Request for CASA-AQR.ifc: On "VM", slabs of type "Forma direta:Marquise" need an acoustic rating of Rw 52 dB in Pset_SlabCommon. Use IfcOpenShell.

First a look at what the model holds.

```python
import ifcopenshell
import ifcopenshell.util.element

model = ifcopenshell.open("CASA-AQR.ifc")
print(model.schema)
storey = next(s for s in model.by_type("IfcBuildingStorey") if s.Name == "VM")
slabs = [e for e in ifcopenshell.util.element.get_decomposition(storey) if e.is_a("IfcSlab")]
seen = {}
for e in slabs:
    element_type = ifcopenshell.util.element.get_type(e)
    key = (element_type.Name if element_type != e and element_type else None, ifcopenshell.util.element.get_pset(e, "Pset_SlabCommon", "AcousticRating"))
    seen[key] = seen.get(key, 0) + 1
for (name, value), count in sorted(seen.items(), key=str):
    print(count, "x", name, "|", value)
```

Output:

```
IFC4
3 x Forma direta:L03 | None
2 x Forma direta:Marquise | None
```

```python
import ifcopenshell
import ifcopenshell.api.pset
import ifcopenshell.util.element

model = ifcopenshell.open("CASA-AQR.ifc")

storey = next(s for s in model.by_type("IfcBuildingStorey") if s.Name == "VM")
slabs = [e for e in ifcopenshell.util.element.get_decomposition(storey) if e.is_a("IfcSlab")]

count = 0
for e in slabs:
    element_type = ifcopenshell.util.element.get_type(e)
    if element_type in (None, e) or element_type.Name != "Forma direta:Marquise":
        continue
    # add_pset returns the element's existing set when there is one.
    pset = ifcopenshell.api.pset.add_pset(model, product=e, name="Pset_SlabCommon")
    ifcopenshell.api.pset.edit_pset(model, pset=pset, properties={"AcousticRating": "Rw 52 dB"})
    count += 1

print(count, "slabs updated")

model.write("CASA-AQR_v2.ifc")
```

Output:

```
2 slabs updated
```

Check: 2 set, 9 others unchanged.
